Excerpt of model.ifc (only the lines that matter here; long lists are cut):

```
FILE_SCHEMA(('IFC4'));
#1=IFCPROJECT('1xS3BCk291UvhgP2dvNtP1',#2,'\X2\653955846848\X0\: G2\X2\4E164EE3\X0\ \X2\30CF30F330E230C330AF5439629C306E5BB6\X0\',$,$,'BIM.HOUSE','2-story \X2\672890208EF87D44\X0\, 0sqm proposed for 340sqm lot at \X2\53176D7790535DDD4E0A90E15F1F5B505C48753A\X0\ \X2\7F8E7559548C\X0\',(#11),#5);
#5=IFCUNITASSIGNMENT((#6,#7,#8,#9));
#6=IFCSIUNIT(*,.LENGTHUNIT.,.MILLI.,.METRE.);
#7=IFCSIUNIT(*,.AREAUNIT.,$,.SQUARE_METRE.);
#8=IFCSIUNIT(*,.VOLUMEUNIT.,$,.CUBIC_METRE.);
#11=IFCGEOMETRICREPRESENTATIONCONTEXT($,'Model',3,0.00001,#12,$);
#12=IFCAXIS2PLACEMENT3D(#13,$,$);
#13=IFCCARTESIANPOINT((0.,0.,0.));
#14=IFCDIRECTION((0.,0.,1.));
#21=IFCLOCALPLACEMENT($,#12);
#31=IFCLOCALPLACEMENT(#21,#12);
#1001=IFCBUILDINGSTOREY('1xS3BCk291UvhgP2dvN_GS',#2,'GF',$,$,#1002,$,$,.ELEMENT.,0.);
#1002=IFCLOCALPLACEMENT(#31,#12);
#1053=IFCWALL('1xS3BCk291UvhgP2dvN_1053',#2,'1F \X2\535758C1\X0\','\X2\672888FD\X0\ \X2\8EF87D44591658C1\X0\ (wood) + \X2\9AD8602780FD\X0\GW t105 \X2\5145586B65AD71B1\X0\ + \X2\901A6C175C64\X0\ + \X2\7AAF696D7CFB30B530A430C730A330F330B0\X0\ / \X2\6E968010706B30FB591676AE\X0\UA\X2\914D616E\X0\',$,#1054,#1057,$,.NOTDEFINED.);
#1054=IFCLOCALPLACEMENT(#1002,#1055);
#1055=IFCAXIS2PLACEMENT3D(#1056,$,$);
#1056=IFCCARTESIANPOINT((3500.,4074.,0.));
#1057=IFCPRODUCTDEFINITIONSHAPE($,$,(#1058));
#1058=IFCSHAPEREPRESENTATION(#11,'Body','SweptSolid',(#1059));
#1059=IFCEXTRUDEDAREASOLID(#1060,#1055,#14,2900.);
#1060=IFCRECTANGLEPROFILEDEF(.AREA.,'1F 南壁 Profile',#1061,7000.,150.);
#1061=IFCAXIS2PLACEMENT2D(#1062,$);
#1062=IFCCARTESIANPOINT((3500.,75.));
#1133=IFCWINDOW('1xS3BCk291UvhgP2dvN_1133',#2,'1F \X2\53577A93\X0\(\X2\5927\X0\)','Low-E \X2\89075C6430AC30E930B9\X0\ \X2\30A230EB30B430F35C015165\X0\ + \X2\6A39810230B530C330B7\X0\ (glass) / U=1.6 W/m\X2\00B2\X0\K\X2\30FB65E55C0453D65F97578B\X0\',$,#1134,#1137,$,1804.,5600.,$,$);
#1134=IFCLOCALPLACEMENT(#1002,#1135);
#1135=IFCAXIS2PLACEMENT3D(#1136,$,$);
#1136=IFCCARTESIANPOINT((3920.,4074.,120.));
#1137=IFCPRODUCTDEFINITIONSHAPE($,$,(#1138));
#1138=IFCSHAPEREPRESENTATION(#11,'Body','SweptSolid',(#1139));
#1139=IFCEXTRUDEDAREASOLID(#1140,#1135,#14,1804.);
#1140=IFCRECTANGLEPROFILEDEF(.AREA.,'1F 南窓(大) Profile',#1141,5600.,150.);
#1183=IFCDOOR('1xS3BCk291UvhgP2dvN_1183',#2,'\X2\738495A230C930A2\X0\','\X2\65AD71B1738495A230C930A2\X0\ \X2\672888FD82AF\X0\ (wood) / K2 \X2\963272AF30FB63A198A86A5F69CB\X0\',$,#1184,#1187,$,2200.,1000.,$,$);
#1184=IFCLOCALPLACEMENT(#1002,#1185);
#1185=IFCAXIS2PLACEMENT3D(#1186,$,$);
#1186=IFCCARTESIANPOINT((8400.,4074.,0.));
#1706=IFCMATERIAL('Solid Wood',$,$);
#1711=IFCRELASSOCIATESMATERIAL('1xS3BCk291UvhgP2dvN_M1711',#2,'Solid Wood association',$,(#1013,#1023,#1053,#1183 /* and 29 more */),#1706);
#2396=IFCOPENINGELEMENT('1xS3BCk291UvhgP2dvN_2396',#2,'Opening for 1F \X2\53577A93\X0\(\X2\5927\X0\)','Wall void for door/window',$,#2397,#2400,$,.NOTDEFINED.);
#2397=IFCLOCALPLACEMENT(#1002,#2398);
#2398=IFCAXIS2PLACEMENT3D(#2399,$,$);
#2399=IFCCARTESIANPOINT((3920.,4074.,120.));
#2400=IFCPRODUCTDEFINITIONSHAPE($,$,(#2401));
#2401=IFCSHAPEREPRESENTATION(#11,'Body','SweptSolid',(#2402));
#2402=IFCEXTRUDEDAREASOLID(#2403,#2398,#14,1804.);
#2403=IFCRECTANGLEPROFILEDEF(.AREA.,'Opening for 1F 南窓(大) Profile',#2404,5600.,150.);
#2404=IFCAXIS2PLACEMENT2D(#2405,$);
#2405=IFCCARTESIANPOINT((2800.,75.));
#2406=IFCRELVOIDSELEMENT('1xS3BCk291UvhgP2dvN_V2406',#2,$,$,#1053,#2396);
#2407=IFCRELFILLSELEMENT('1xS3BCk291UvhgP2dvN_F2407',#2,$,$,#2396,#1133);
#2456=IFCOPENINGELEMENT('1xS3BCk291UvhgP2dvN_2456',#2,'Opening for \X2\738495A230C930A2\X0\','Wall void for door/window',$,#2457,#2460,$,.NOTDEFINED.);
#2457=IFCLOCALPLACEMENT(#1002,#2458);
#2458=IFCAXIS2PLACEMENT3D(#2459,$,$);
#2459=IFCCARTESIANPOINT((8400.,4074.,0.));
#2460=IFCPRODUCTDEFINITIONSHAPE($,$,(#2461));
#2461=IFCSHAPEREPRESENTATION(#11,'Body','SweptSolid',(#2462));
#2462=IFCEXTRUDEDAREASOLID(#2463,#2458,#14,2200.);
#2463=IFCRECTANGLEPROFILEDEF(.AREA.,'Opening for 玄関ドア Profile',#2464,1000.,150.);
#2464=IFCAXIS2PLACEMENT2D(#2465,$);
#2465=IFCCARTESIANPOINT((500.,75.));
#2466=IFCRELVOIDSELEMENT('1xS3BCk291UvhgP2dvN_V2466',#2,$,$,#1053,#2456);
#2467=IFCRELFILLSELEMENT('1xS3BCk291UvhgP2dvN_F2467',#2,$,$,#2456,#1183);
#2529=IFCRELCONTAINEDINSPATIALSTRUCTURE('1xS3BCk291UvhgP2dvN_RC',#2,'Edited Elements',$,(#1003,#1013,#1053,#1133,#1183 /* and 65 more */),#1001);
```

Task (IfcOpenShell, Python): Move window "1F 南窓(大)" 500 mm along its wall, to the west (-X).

```python
import ifcopenshell
import ifcopenshell.api.geometry
import ifcopenshell.util.placement

model = ifcopenshell.open("model.ifc")

window = model.by_id(1133)
opening = window.FillsVoids[0].RelatingOpeningElement
wall = opening.VoidsElements[0].RelatingBuildingElement

wall_matrix = ifcopenshell.util.placement.get_local_placement(wall.ObjectPlacement)
shift = wall_matrix[:3, 0] * -500.0
before = ifcopenshell.util.placement.get_local_placement(window.ObjectPlacement)[:3, 3].copy()

# The window is not placed relative to its opening, so move both.
for product in (opening, window):
    matrix = ifcopenshell.util.placement.get_local_placement(product.ObjectPlacement)
    matrix[:3, 3] += shift
    ifcopenshell.api.geometry.edit_object_placement(model, product=product, matrix=matrix, is_si=False)

after = ifcopenshell.util.placement.get_local_placement(window.ObjectPlacement)[:3, 3]
print("window moved by", (after - before).round(3) + 0.0)

model.write("model_updated.ifc")
```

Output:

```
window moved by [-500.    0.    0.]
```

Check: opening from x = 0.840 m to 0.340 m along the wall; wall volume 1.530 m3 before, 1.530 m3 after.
